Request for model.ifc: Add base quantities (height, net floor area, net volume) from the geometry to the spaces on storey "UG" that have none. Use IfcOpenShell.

First a look at what the model holds.

```python
import ifcopenshell
import ifcopenshell.util.element
import ifcopenshell.util.unit

model = ifcopenshell.open("model.ifc")
print(model.schema)
for unit_type in ("LENGTHUNIT", "AREAUNIT", "VOLUMEUNIT"):
    print(unit_type, ifcopenshell.util.unit.calculate_unit_scale(model, unit_type))
storey = next(s for s in model.by_type("IfcBuildingStorey") if s.Name == "UG")
spaces = [e for e in ifcopenshell.util.element.get_decomposition(storey) if e.is_a("IfcSpace")]
for e in sorted(spaces, key=lambda e: e.id()):
    print(e.id(), e.is_a(), e.Name, list(ifcopenshell.util.element.get_psets(e, qtos_only=True)), sep=" | ")
```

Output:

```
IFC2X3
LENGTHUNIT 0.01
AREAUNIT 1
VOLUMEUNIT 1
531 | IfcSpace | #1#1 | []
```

```python
import ifcopenshell
import ifcopenshell.api.pset
import ifcopenshell.geom
import ifcopenshell.util.element
import ifcopenshell.util.shape
import ifcopenshell.util.unit

model = ifcopenshell.open("model.ifc")
unit_scale = ifcopenshell.util.unit.calculate_unit_scale(model)
area_scale = ifcopenshell.util.unit.calculate_unit_scale(model, "AREAUNIT")
volume_scale = ifcopenshell.util.unit.calculate_unit_scale(model, "VOLUMEUNIT")
settings = ifcopenshell.geom.settings()

storey = next(s for s in model.by_type("IfcBuildingStorey") if s.Name == "UG")
spaces = [e for e in ifcopenshell.util.element.get_decomposition(storey) if e.is_a("IfcSpace")]

for e in sorted(spaces, key=lambda e: e.id()):
    if ifcopenshell.util.element.get_psets(e, qtos_only=True, should_inherit=False):
        continue
    # Geometry comes back in metres, in the element's own axes.
    shape = ifcopenshell.geom.create_shape(settings, e)
    values = {
        "Height": ifcopenshell.util.shape.get_z(shape.geometry) / unit_scale,
        "NetFloorArea": ifcopenshell.util.shape.get_footprint_area(shape.geometry) / area_scale,
        "NetVolume": ifcopenshell.util.shape.get_volume(shape.geometry) / volume_scale,
    }
    qto = ifcopenshell.api.pset.add_qto(model, product=e, name="BaseQuantities")
    ifcopenshell.api.pset.edit_qto(model, qto=qto, properties=values)
    print(e.id(), {k: round(v, 3) for k, v in values.items()})

model.write("model_rev.ifc")
```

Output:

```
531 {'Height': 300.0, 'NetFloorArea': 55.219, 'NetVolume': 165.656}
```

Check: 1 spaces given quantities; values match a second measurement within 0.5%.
